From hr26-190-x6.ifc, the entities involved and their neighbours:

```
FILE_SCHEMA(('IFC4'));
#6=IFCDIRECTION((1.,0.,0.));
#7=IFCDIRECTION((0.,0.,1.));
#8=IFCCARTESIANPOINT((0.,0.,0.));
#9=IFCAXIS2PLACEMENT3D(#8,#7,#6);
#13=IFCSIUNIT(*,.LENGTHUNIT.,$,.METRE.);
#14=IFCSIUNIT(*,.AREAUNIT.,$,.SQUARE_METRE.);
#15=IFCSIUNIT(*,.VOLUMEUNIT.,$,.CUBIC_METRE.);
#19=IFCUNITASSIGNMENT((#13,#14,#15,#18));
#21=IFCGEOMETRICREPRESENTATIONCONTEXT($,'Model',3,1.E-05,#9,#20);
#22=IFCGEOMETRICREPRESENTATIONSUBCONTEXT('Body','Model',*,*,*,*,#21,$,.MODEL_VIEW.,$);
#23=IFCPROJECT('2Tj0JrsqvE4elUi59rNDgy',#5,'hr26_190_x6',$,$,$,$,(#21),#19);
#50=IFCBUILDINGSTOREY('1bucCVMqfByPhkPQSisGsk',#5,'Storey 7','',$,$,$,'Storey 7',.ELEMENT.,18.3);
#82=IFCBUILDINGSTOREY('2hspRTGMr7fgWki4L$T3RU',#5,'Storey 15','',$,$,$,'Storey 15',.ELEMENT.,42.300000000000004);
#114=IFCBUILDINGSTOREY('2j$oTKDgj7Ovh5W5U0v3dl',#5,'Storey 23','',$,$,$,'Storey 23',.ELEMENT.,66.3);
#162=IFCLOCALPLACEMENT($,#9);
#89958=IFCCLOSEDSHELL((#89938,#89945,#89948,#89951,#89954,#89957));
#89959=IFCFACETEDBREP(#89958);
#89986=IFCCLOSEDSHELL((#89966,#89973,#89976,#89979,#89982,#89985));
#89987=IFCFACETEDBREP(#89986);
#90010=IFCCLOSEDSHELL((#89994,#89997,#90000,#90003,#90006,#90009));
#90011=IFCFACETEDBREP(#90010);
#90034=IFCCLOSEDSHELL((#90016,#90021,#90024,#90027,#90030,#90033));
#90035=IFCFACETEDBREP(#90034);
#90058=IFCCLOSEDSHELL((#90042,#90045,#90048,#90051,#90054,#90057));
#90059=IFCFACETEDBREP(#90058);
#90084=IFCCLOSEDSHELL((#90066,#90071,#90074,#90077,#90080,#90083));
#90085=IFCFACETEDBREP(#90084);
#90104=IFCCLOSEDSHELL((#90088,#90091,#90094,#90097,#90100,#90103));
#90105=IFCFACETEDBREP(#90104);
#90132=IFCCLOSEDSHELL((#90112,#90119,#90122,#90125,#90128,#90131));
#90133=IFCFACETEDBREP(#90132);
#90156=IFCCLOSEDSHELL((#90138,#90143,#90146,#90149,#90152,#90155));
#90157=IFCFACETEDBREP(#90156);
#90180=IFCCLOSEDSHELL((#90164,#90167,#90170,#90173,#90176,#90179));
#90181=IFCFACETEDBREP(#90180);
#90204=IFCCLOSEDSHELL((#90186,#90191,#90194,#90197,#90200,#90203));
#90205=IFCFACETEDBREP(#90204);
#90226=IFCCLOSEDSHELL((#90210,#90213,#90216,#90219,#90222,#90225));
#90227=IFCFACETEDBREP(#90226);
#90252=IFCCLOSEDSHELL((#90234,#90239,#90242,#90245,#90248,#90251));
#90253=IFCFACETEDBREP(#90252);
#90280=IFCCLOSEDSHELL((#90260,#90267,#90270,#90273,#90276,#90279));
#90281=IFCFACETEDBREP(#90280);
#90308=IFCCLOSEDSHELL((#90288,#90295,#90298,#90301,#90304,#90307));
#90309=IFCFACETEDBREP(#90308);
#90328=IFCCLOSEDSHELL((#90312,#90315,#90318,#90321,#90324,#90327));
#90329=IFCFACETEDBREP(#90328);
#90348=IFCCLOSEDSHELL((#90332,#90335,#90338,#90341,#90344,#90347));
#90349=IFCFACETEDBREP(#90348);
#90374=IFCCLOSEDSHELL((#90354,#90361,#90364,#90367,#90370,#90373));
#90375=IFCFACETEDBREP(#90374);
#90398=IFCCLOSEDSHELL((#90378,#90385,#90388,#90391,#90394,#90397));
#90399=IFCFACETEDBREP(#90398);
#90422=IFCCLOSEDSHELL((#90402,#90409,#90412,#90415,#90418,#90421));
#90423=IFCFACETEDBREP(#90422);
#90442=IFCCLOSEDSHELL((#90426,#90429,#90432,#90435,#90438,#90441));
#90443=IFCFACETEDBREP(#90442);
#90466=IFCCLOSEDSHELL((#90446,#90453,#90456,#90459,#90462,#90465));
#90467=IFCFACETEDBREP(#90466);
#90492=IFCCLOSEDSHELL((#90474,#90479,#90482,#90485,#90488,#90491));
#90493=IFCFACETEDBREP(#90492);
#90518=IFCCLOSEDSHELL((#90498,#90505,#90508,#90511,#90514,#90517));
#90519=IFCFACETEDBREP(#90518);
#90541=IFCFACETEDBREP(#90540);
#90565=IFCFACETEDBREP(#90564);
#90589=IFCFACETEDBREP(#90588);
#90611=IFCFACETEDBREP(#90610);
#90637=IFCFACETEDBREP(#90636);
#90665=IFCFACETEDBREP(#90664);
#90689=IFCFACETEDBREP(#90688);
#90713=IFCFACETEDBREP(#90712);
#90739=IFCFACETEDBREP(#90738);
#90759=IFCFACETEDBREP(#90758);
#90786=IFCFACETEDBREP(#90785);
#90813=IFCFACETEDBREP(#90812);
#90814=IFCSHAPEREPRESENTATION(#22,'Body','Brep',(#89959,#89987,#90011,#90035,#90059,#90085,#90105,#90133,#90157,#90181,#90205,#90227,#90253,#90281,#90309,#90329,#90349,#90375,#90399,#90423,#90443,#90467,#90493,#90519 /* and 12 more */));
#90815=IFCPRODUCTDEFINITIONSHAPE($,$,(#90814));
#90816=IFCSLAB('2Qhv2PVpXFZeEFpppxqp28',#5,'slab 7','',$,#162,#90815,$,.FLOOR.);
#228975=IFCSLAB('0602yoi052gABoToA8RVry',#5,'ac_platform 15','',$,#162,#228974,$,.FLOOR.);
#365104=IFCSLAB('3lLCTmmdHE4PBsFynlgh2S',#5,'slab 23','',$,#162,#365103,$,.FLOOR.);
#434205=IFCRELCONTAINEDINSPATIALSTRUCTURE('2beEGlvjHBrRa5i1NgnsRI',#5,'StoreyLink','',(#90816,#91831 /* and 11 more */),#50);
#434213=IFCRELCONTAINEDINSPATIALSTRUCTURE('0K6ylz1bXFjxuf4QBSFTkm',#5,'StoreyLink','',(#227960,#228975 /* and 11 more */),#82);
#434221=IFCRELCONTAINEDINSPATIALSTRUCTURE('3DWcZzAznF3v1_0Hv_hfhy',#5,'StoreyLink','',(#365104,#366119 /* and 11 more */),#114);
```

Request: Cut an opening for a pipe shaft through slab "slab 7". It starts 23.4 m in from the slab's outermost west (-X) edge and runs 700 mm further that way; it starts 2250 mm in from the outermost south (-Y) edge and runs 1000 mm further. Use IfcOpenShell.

```python
import numpy as np
import ifcopenshell
import ifcopenshell.api.feature
import ifcopenshell.api.geometry
import ifcopenshell.api.root
import ifcopenshell.geom
import ifcopenshell.util.placement
import ifcopenshell.util.representation
import ifcopenshell.util.shape
import ifcopenshell.util.unit

model = ifcopenshell.open("hr26-190-x6.ifc")
unit_scale = ifcopenshell.util.unit.calculate_unit_scale(model)
settings = ifcopenshell.geom.settings()


def volume(element):
    """Net volume in cubic metres, openings subtracted."""
    shape = ifcopenshell.geom.create_shape(settings, element)
    return ifcopenshell.util.shape.get_volume(shape.geometry)


slab = model.by_guid("2Qhv2PVpXFZeEFpppxqp28")
before = volume(slab)

# Extent in the slab's own axes, in metres. The edges named are its -X and -Y sides.
slab_shape = ifcopenshell.geom.create_shape(settings, slab)
vertices = ifcopenshell.util.shape.get_vertices(slab_shape.geometry)
x_min, y_min, bottom = vertices.min(axis=0)
top = vertices[:, 2].max()

opening = ifcopenshell.api.root.create_entity(model, ifc_class="IfcOpeningElement", name="Pipe shaft opening", predefined_type="OPENING")
context = ifcopenshell.util.representation.get_context(model, "Model", "Body", "MODEL_VIEW")
width, depth = 0.7, 1
outline = [(0.0, 0.0), (width, 0.0), (width, depth), (0.0, depth), (0.0, 0.0)]
# Overshoot both faces by 50 mm so the cut is clean.
shape = ifcopenshell.api.geometry.add_slab_representation(
    model, context=context, depth=top - bottom + 0.1, polyline=outline
)
ifcopenshell.api.geometry.assign_representation(model, product=opening, representation=shape)

matrix = ifcopenshell.util.placement.get_local_placement(slab.ObjectPlacement)
matrix[:, 3] = matrix @ np.append(np.array([x_min + 23.4, y_min + 2.25, bottom - 0.05]) / unit_scale, 1.0)
ifcopenshell.api.geometry.edit_object_placement(model, product=opening, matrix=matrix, is_si=False)
ifcopenshell.api.feature.add_feature(model, feature=opening, element=slab)

after = volume(slab)

print(f"slab volume {before:.3f} -> {after:.3f} m3")

model.write("hr26-190-x6_rev.ifc")
```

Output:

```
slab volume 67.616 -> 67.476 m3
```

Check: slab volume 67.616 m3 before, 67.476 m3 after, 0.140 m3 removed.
